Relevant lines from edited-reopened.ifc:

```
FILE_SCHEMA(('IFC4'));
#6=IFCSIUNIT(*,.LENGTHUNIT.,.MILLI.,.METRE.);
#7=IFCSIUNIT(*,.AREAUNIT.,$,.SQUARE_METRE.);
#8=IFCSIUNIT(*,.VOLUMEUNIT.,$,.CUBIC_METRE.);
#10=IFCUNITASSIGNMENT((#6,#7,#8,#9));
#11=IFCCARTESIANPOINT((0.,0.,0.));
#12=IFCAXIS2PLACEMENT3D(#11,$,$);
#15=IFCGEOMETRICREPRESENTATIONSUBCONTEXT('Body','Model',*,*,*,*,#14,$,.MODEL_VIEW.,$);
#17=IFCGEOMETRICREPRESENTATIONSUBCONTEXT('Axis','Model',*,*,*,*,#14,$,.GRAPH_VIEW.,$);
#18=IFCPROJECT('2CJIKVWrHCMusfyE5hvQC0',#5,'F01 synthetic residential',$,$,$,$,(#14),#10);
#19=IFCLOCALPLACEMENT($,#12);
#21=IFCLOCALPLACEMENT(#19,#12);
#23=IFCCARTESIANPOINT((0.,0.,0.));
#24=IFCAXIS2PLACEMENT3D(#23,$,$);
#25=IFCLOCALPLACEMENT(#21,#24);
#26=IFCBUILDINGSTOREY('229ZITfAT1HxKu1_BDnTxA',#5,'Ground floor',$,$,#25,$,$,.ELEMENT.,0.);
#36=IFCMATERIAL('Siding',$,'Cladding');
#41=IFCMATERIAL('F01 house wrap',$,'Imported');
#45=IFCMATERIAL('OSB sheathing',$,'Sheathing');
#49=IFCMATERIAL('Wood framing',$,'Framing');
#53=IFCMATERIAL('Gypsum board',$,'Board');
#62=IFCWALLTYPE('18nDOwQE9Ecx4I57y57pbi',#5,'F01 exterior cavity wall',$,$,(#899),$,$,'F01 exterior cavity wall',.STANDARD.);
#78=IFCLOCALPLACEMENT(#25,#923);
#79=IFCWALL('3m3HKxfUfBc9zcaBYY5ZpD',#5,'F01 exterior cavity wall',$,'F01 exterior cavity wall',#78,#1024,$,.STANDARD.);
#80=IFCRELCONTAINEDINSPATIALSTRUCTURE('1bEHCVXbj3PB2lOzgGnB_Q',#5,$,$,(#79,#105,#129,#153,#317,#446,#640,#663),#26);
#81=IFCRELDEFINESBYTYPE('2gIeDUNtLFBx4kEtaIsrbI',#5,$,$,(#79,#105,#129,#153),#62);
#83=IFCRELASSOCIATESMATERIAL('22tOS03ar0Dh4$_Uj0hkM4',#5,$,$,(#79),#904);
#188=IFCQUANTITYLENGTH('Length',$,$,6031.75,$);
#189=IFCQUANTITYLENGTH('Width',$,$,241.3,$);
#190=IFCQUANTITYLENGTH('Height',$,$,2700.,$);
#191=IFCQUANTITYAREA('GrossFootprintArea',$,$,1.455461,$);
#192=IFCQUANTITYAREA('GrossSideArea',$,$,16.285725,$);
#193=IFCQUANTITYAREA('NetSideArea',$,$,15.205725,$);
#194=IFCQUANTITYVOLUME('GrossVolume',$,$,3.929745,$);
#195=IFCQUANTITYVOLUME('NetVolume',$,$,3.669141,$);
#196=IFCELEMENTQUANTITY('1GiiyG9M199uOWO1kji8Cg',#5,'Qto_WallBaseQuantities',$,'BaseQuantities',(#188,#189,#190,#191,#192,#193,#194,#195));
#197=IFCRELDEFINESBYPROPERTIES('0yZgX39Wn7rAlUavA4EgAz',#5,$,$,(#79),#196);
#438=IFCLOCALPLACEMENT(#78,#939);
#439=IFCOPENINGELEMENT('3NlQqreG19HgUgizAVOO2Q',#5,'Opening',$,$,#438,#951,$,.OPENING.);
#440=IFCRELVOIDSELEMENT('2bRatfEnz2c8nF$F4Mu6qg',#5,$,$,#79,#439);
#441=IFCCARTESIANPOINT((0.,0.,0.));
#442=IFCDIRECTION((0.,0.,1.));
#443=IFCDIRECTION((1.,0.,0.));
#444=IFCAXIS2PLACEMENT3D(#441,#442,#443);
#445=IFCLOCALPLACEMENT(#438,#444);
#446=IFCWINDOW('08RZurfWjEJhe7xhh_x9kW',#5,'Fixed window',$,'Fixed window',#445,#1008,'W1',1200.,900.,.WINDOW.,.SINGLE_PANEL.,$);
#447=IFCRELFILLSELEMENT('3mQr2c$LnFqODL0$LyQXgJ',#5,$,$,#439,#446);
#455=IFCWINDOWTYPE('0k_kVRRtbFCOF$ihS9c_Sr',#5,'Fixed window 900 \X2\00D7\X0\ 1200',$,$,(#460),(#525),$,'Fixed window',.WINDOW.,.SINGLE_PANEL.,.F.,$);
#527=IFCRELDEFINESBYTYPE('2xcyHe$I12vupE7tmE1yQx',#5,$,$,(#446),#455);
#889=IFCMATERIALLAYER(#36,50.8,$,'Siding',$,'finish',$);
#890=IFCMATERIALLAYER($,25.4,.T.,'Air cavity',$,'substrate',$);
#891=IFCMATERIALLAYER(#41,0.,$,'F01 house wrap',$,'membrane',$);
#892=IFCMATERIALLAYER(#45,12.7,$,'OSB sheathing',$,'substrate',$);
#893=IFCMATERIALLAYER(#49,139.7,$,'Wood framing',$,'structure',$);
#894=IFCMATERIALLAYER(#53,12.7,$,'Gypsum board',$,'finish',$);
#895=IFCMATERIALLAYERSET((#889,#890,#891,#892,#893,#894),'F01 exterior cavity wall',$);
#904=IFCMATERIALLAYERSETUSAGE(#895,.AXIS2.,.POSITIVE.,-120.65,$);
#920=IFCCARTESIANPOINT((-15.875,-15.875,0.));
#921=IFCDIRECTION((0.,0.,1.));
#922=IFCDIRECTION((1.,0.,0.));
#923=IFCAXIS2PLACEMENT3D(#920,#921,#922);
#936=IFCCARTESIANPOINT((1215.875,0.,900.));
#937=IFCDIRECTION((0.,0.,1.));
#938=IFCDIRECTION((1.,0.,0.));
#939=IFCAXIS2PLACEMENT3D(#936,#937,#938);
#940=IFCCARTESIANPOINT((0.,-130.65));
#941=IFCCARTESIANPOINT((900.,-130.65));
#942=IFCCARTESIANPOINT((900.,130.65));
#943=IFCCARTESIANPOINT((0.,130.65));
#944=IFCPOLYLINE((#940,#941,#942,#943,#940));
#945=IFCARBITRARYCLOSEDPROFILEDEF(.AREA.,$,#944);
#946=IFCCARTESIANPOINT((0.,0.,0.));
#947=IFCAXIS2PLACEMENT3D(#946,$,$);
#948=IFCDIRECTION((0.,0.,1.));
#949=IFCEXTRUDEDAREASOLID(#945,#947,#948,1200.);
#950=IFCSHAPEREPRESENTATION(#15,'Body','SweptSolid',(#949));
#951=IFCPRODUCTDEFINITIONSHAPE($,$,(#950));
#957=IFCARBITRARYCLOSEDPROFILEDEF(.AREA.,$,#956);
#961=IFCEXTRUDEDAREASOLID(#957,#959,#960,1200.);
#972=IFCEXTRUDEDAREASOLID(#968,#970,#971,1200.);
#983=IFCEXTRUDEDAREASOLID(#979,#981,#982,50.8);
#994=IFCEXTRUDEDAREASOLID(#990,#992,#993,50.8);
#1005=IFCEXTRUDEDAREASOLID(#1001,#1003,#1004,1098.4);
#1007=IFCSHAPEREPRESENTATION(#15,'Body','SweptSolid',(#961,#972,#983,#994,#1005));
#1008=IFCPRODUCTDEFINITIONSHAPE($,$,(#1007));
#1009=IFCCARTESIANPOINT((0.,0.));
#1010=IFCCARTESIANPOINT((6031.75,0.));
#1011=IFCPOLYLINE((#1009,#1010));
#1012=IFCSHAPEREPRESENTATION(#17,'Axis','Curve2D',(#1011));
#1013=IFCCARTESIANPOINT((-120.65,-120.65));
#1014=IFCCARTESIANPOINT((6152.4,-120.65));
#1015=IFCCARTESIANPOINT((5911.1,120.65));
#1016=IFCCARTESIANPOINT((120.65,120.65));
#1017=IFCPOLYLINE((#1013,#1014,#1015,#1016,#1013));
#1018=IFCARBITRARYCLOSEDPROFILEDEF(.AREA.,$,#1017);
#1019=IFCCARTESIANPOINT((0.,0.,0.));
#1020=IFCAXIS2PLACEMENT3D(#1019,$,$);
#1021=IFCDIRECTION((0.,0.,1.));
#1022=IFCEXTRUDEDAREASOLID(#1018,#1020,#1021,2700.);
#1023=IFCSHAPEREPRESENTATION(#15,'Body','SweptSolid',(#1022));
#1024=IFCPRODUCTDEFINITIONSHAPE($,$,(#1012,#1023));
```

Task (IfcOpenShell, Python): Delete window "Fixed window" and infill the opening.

```python
import ifcopenshell
import ifcopenshell.api.feature
import ifcopenshell.api.pset
import ifcopenshell.api.root
import ifcopenshell.geom
import ifcopenshell.util.element
import ifcopenshell.util.shape
import ifcopenshell.util.unit

model = ifcopenshell.open("edited-reopened.ifc")
area_scale = ifcopenshell.util.unit.calculate_unit_scale(model, "AREAUNIT")
volume_scale = ifcopenshell.util.unit.calculate_unit_scale(model, "VOLUMEUNIT")
settings = ifcopenshell.geom.settings()


def volume(element):
    """Net volume in cubic metres, openings subtracted."""
    shape = ifcopenshell.geom.create_shape(settings, element)
    return ifcopenshell.util.shape.get_volume(shape.geometry)


window = model.by_guid("08RZurfWjEJhe7xhh_x9kW")
opening = window.FillsVoids[0].RelatingOpeningElement
wall = opening.VoidsElements[0].RelatingBuildingElement
before = volume(wall)

ifcopenshell.api.root.remove_product(model, product=window)
ifcopenshell.api.feature.remove_feature(model, feature=opening)

after = volume(wall)
thickness = 0.2413  # wall thickness in metres

# Update the wall's stored quantities.
qto = model.by_id(ifcopenshell.util.element.get_pset(wall, "Qto_WallBaseQuantities", should_inherit=False)["id"])
ifcopenshell.api.pset.edit_qto(model, qto=qto, properties={
    "NetSideArea": after / thickness / area_scale,
    "NetVolume": after / volume_scale,
})

print(f"wall volume {before:.3f} -> {after:.3f} m3")

model.write("edited-reopened-out.ifc")
```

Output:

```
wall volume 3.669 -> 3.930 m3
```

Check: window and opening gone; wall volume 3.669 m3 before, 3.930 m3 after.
